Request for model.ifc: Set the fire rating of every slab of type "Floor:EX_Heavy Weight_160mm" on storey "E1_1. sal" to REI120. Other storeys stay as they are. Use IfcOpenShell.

First a look at what the model holds.

```python
import ifcopenshell
import ifcopenshell.util.element

model = ifcopenshell.open("model.ifc")
print(model.schema)
storey = next(s for s in model.by_type("IfcBuildingStorey") if s.Name == "E1_1. sal")
slabs = [e for e in ifcopenshell.util.element.get_decomposition(storey) if e.is_a("IfcSlab")]
seen = {}
for e in slabs:
    element_type = ifcopenshell.util.element.get_type(e)
    key = (element_type.Name if element_type != e and element_type else None, ifcopenshell.util.element.get_pset(e, "Pset_SlabCommon", "FireRating"))
    seen[key] = seen.get(key, 0) + 1
for (name, value), count in sorted(seen.items(), key=str):
    print(count, "x", name, "|", value)
```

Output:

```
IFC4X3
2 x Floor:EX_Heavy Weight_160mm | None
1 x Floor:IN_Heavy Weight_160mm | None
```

```python
import ifcopenshell
import ifcopenshell.api.pset
import ifcopenshell.util.element

model = ifcopenshell.open("model.ifc")

storey = next(s for s in model.by_type("IfcBuildingStorey") if s.Name == "E1_1. sal")
slabs = [e for e in ifcopenshell.util.element.get_decomposition(storey) if e.is_a("IfcSlab")]

count = 0
for e in slabs:
    element_type = ifcopenshell.util.element.get_type(e)
    if element_type in (None, e) or element_type.Name != "Floor:EX_Heavy Weight_160mm":
        continue
    # add_pset returns the element's existing set when there is one.
    pset = ifcopenshell.api.pset.add_pset(model, product=e, name="Pset_SlabCommon")
    ifcopenshell.api.pset.edit_pset(model, pset=pset, properties={"FireRating": "REI120"})
    count += 1

print(count, "slabs updated")

model.write("model_v2.ifc")
```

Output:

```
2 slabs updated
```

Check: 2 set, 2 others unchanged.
